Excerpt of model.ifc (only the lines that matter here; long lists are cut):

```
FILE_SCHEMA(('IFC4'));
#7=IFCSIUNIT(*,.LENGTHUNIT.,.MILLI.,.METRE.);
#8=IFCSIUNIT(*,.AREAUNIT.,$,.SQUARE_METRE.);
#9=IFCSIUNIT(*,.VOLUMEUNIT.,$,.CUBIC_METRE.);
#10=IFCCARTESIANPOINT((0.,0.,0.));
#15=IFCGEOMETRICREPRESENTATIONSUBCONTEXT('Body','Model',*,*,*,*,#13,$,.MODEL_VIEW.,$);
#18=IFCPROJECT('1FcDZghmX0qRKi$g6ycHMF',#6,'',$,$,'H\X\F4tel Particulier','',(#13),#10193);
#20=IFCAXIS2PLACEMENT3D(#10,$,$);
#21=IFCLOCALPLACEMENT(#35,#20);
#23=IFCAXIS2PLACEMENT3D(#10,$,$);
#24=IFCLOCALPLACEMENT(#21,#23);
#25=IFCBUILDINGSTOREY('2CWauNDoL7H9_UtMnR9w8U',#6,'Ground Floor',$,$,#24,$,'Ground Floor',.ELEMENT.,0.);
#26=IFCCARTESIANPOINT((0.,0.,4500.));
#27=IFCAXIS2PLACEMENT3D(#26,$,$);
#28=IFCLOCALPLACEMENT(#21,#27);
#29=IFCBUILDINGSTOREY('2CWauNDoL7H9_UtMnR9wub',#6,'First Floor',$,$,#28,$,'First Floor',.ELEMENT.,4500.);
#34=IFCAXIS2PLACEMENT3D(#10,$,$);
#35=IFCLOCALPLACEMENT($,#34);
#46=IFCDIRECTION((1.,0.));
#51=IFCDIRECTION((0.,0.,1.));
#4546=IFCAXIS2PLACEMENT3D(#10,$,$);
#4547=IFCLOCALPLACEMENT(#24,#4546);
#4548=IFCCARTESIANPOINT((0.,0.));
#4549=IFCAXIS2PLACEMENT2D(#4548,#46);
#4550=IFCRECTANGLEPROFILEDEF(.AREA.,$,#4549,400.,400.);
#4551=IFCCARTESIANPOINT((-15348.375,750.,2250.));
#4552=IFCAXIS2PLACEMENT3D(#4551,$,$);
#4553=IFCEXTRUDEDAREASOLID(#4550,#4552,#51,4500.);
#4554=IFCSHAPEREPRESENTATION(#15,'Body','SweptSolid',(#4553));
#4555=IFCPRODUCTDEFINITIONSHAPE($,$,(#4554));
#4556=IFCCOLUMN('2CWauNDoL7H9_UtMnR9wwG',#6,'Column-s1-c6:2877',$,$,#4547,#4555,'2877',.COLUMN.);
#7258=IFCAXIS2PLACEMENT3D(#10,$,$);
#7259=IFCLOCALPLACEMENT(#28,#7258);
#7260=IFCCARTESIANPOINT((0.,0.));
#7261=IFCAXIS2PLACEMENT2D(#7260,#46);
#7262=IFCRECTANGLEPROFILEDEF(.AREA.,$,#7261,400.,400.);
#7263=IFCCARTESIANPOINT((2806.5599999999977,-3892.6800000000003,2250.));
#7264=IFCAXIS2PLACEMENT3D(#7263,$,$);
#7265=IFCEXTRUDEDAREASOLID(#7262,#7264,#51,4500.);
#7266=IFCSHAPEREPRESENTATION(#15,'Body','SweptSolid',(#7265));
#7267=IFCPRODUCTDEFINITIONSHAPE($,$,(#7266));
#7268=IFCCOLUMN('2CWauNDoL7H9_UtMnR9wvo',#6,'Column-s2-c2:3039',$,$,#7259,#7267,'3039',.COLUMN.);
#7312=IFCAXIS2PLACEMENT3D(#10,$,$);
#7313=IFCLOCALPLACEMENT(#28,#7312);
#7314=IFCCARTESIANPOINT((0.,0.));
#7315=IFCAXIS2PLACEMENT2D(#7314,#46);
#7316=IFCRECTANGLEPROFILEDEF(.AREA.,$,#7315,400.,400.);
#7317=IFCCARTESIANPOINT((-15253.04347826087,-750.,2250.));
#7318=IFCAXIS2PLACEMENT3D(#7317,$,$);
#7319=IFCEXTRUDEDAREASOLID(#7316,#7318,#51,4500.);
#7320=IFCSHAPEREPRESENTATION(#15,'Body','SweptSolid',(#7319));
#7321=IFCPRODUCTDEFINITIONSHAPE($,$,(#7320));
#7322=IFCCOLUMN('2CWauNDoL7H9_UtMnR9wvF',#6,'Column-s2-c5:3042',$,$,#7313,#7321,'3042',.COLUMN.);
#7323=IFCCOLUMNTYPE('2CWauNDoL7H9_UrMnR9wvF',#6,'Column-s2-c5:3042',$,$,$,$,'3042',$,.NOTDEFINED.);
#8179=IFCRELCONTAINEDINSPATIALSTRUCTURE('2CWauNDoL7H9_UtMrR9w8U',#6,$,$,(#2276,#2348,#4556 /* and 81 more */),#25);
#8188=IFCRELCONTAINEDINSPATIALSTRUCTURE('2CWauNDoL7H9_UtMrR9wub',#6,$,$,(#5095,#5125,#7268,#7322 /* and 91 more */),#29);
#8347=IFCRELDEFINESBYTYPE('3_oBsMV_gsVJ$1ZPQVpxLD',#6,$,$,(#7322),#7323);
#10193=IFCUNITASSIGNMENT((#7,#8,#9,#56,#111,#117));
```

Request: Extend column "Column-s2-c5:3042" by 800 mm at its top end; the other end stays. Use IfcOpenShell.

```python
import ifcopenshell
import ifcopenshell.util.representation

model = ifcopenshell.open("model.ifc")

member = model.by_id(7322)
change = 800.0

# The extrusion runs towards the end named, so only its depth changes.
body = ifcopenshell.util.representation.get_representation(member, "Model", "Body")
solid = body.Items[0]
old_length = solid.Depth
solid.Depth += change

print(f"length {old_length:g} -> {solid.Depth:g}")

model.write("model_edited.ifc")
```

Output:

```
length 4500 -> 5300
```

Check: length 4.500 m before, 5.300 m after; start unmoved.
